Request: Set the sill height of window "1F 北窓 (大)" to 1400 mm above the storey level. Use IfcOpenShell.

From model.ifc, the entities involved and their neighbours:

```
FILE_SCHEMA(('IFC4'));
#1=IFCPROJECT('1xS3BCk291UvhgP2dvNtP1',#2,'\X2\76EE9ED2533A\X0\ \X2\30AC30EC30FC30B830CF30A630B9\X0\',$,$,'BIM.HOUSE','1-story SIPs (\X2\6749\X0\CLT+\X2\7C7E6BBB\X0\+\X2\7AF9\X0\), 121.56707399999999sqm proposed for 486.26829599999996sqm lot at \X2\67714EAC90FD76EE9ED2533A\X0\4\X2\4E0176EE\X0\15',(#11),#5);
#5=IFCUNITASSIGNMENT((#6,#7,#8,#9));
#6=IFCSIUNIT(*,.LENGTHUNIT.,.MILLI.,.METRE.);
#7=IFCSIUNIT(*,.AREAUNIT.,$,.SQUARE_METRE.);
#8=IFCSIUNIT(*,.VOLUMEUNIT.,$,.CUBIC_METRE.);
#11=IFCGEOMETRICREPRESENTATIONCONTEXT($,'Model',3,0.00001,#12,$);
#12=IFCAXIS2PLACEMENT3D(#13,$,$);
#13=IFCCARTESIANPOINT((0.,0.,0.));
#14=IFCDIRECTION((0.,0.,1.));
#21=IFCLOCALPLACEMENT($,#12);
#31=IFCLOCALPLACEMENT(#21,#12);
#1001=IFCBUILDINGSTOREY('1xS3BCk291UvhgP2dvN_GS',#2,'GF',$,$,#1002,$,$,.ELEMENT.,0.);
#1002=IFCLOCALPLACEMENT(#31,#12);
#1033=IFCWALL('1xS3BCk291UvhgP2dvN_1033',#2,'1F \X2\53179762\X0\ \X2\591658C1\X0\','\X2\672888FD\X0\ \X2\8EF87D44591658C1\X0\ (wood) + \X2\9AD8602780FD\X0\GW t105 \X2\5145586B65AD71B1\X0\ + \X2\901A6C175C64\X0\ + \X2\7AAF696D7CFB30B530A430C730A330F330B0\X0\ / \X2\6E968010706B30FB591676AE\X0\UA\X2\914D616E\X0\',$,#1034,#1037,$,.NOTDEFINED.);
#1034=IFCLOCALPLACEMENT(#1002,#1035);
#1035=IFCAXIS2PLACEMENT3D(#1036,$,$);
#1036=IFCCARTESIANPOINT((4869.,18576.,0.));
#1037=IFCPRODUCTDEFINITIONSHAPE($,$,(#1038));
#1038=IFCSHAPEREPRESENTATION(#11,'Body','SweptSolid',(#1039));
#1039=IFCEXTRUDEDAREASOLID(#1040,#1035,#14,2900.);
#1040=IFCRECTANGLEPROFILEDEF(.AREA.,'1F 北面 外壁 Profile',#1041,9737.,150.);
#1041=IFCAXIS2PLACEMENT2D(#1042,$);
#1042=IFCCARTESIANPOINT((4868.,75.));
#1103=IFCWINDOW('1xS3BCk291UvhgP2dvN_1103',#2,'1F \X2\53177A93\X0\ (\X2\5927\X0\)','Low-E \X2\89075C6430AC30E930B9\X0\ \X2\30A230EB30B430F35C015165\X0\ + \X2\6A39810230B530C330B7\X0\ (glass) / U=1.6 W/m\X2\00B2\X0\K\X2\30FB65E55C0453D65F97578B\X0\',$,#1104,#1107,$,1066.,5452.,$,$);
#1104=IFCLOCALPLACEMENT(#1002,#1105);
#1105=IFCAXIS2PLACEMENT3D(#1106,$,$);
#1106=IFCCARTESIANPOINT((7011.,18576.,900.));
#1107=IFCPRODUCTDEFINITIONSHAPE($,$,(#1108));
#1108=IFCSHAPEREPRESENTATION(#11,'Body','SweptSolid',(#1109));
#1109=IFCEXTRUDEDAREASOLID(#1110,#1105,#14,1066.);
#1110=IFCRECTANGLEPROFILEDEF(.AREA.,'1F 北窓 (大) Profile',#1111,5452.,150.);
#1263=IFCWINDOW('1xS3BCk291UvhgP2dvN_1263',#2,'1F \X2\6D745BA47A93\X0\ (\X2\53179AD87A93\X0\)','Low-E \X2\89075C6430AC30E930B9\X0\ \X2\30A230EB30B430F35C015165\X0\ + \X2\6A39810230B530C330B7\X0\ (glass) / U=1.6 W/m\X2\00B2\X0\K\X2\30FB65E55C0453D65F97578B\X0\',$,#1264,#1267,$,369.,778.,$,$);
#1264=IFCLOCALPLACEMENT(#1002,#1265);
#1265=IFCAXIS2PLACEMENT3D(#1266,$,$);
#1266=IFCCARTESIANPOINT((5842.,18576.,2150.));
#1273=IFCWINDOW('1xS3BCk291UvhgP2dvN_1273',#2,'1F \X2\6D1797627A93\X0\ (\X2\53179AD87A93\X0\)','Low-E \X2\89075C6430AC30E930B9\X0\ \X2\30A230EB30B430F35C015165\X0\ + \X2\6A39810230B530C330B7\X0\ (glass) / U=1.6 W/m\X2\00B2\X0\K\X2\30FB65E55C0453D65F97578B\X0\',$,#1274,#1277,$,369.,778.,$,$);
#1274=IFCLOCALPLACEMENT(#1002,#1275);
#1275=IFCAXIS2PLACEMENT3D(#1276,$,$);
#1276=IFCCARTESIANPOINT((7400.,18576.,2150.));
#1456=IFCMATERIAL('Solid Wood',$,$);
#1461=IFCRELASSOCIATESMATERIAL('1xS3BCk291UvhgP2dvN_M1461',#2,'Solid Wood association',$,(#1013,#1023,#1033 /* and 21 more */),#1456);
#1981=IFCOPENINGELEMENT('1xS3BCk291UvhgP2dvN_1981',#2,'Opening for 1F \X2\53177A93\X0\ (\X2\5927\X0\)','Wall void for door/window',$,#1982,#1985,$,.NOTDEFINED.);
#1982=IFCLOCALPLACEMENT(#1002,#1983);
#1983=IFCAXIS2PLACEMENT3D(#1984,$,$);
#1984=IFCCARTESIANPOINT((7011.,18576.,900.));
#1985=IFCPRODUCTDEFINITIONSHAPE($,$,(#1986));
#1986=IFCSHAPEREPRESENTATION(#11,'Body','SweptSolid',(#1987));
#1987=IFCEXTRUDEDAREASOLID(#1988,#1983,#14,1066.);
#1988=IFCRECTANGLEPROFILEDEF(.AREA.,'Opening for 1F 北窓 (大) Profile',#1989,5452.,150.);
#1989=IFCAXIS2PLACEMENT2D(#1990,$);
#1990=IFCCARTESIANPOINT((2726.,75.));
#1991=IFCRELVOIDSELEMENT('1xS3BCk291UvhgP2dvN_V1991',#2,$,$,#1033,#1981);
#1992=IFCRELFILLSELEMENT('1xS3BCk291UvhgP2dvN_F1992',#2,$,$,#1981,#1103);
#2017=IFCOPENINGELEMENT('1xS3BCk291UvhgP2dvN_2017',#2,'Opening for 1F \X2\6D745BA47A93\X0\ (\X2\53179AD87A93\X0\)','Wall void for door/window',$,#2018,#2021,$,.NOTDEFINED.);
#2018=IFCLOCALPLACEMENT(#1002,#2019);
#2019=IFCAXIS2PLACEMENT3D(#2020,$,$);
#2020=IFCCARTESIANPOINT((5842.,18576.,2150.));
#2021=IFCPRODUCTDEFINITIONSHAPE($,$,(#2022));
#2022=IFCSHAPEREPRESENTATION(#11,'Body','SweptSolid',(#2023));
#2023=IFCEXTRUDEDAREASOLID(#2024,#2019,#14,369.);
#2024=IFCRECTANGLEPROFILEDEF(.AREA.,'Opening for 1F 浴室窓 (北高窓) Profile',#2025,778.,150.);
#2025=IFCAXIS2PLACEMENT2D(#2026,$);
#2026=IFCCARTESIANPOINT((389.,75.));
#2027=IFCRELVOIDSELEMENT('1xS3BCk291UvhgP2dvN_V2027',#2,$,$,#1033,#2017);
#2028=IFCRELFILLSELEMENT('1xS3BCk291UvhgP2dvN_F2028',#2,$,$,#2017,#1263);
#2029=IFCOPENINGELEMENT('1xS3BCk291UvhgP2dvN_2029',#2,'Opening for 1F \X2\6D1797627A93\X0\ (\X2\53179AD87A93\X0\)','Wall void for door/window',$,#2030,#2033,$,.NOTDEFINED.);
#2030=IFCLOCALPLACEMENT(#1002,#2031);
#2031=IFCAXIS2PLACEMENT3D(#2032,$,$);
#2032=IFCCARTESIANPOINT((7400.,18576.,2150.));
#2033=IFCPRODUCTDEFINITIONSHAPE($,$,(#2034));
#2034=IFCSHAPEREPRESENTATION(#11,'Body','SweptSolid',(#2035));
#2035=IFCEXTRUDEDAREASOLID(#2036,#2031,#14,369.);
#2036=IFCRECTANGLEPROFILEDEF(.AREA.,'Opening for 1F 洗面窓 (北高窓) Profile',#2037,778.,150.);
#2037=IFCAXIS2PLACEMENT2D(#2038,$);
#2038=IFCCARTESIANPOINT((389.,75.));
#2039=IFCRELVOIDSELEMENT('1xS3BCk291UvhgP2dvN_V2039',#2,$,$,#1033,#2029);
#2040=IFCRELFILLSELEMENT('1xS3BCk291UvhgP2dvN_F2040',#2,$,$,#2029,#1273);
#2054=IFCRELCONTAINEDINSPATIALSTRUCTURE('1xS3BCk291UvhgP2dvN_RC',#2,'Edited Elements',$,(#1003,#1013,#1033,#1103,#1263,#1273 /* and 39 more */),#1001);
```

```python
import numpy as np
import ifcopenshell
import ifcopenshell.api.geometry
import ifcopenshell.geom
import ifcopenshell.util.element
import ifcopenshell.util.placement
import ifcopenshell.util.shape
import ifcopenshell.util.unit

model = ifcopenshell.open("model.ifc")
unit_scale = ifcopenshell.util.unit.calculate_unit_scale(model)

window = model.by_guid("1xS3BCk291UvhgP2dvN_1103")
opening = window.FillsVoids[0].RelatingOpeningElement
storey = ifcopenshell.util.element.get_container(window, ifc_class="IfcBuildingStorey")
level = ifcopenshell.util.placement.get_local_placement(storey.ObjectPlacement)[2, 3]

# The opening's origin need not be at the sill, so measure its lowest point.
shape = ifcopenshell.geom.create_shape(ifcopenshell.geom.settings(), opening)
bottom = ifcopenshell.util.shape.get_shape_bottom_elevation(shape, shape.geometry) / unit_scale
dz = level + 1.4 / unit_scale - bottom

shift = np.array([0.0, 0.0, dz])
# The window is not placed relative to its opening, so move both.
for product in (opening, window):
    matrix = ifcopenshell.util.placement.get_local_placement(product.ObjectPlacement)
    matrix[:3, 3] += shift
    ifcopenshell.api.geometry.edit_object_placement(model, product=product, matrix=matrix, is_si=False)

print(f"moved by {dz * unit_scale:+.3f} m")

model.write("model_edited.ifc")
```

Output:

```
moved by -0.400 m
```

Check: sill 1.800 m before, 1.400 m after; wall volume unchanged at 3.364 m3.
